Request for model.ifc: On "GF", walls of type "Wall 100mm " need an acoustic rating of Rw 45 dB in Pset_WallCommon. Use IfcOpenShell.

First a look at what the model holds.

```python
import ifcopenshell
import ifcopenshell.util.element

model = ifcopenshell.open("model.ifc")
print(model.schema)
storey = next(s for s in model.by_type("IfcBuildingStorey") if s.Name == "GF")
walls = [e for e in ifcopenshell.util.element.get_decomposition(storey) if e.is_a("IfcWall")]
seen = {}
for e in walls:
    element_type = ifcopenshell.util.element.get_type(e)
    key = (element_type.Name if element_type != e and element_type else None, ifcopenshell.util.element.get_pset(e, "Pset_WallCommon", "AcousticRating"))
    seen[key] = seen.get(key, 0) + 1
for (name, value), count in sorted(seen.items(), key=str):
    print(count, "x", name, "|", value)
```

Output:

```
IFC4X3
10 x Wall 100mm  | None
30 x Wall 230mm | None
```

```python
import ifcopenshell
import ifcopenshell.api.pset
import ifcopenshell.util.element

model = ifcopenshell.open("model.ifc")

storey = next(s for s in model.by_type("IfcBuildingStorey") if s.Name == "GF")
walls = [e for e in ifcopenshell.util.element.get_decomposition(storey) if e.is_a("IfcWall")]

count = 0
for e in walls:
    element_type = ifcopenshell.util.element.get_type(e)
    if element_type in (None, e) or element_type.Name != "Wall 100mm ":
        continue
    # add_pset returns the element's existing set when there is one.
    pset = ifcopenshell.api.pset.add_pset(model, product=e, name="Pset_WallCommon")
    ifcopenshell.api.pset.edit_pset(model, pset=pset, properties={"AcousticRating": "Rw 45 dB"})
    count += 1

print(count, "walls updated")

model.write("model_edited.ifc")
```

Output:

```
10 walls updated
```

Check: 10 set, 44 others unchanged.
